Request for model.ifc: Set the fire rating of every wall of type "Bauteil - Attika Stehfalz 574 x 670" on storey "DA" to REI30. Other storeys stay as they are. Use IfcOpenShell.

First a look at what the model holds.

```python
import ifcopenshell
import ifcopenshell.util.element

model = ifcopenshell.open("model.ifc")
print(model.schema)
storey = next(s for s in model.by_type("IfcBuildingStorey") if s.Name == "DA")
walls = [e for e in ifcopenshell.util.element.get_decomposition(storey) if e.is_a("IfcWall")]
seen = {}
for e in walls:
    element_type = ifcopenshell.util.element.get_type(e)
    key = (element_type.Name if element_type != e and element_type else None, ifcopenshell.util.element.get_pset(e, "Pset_WallCommon", "FireRating"))
    seen[key] = seen.get(key, 0) + 1
for (name, value), count in sorted(seen.items(), key=str):
    print(count, "x", name, "|", value)
```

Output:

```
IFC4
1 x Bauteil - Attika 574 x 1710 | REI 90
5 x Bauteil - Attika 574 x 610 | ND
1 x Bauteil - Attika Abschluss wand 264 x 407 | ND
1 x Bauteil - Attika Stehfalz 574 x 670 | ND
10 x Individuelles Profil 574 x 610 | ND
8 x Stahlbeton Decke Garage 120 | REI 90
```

```python
import ifcopenshell
import ifcopenshell.api.pset
import ifcopenshell.util.element

model = ifcopenshell.open("model.ifc")

storey = next(s for s in model.by_type("IfcBuildingStorey") if s.Name == "DA")
walls = [e for e in ifcopenshell.util.element.get_decomposition(storey) if e.is_a("IfcWall")]

count = 0
for e in walls:
    element_type = ifcopenshell.util.element.get_type(e)
    if element_type in (None, e) or element_type.Name != "Bauteil - Attika Stehfalz 574 x 670":
        continue
    # add_pset returns the element's existing set when there is one.
    pset = ifcopenshell.api.pset.add_pset(model, product=e, name="Pset_WallCommon")
    ifcopenshell.api.pset.edit_pset(model, pset=pset, properties={"FireRating": "REI30"})
    count += 1

print(count, "walls updated")

model.write("model-out.ifc")
```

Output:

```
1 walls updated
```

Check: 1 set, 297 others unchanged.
